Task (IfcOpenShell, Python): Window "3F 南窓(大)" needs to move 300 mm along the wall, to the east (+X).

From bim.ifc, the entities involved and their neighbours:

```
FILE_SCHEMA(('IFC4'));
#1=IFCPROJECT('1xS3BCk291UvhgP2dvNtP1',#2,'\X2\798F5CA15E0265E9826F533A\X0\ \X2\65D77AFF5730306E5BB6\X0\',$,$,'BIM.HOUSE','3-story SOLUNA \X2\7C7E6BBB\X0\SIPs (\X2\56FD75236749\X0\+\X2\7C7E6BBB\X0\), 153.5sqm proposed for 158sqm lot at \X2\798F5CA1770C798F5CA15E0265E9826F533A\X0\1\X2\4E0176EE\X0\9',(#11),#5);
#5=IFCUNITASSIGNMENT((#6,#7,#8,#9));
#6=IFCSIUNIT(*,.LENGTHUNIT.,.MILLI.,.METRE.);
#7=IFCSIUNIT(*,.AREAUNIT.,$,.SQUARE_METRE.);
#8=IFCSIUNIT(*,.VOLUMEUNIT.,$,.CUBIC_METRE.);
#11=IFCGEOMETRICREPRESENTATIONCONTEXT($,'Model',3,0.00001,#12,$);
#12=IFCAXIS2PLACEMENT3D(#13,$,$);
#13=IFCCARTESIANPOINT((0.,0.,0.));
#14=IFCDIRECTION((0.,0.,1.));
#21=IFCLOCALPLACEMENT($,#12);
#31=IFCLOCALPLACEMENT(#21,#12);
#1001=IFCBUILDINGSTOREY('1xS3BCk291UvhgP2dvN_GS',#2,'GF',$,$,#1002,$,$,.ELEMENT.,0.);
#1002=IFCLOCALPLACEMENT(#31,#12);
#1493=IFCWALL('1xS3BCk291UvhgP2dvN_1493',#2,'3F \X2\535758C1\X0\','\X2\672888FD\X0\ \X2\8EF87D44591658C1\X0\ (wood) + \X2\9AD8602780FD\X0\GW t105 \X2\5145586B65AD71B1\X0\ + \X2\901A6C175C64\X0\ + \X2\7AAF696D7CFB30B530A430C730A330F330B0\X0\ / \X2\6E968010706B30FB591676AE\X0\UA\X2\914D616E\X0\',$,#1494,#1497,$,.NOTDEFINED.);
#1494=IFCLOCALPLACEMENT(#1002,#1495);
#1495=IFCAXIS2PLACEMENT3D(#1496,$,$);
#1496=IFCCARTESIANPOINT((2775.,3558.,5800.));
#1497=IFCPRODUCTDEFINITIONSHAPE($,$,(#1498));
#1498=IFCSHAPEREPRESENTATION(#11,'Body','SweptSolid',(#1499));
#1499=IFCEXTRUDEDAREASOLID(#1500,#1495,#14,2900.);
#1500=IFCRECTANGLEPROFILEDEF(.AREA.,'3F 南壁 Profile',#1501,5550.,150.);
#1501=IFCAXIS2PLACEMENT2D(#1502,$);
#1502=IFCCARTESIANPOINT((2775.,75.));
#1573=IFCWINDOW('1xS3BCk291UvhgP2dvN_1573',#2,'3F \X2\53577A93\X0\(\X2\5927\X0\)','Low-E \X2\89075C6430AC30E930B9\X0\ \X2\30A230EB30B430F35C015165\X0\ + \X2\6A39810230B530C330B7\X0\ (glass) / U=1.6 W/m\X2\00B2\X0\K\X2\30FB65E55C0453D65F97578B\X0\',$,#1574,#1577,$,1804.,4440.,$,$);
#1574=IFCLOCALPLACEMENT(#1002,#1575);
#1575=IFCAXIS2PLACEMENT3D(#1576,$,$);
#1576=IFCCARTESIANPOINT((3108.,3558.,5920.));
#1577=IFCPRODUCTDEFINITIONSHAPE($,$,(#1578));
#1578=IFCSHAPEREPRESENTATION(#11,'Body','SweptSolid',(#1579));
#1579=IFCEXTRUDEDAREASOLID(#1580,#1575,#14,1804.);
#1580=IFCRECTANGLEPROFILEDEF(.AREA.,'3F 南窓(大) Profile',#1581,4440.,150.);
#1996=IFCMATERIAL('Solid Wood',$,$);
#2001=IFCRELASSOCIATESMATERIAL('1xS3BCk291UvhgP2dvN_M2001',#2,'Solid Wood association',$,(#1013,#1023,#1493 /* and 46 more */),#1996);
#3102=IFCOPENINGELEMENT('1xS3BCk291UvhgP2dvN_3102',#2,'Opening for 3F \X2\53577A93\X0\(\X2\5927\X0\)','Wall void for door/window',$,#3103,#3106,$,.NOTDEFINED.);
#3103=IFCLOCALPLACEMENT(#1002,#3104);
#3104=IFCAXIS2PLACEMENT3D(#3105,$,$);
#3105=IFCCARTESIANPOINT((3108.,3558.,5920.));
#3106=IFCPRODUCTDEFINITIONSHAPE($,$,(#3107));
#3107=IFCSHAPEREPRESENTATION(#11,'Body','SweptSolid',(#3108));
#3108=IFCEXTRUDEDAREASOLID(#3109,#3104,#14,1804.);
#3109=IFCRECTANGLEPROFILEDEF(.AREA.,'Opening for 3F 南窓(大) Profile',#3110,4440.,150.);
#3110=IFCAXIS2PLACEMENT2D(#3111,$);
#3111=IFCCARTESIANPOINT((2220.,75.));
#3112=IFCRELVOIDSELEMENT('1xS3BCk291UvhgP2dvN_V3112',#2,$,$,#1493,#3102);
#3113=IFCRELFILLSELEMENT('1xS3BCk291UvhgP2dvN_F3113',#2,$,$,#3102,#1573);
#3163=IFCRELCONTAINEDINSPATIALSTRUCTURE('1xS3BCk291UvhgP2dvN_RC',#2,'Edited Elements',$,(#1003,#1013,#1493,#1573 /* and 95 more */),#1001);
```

```python
import ifcopenshell
import ifcopenshell.api.geometry
import ifcopenshell.util.placement
import ifcopenshell.util.unit

model = ifcopenshell.open("bim.ifc")
unit_scale = ifcopenshell.util.unit.calculate_unit_scale(model)

window = model.by_guid("1xS3BCk291UvhgP2dvN_1573")
opening = window.FillsVoids[0].RelatingOpeningElement
wall = opening.VoidsElements[0].RelatingBuildingElement

wall_matrix = ifcopenshell.util.placement.get_local_placement(wall.ObjectPlacement)
shift = wall_matrix[:3, 0] * 0.3 / unit_scale
before = ifcopenshell.util.placement.get_local_placement(window.ObjectPlacement)[:3, 3].copy()

# The window is not placed relative to its opening, so move both.
for product in (opening, window):
    matrix = ifcopenshell.util.placement.get_local_placement(product.ObjectPlacement)
    matrix[:3, 3] += shift
    ifcopenshell.api.geometry.edit_object_placement(model, product=product, matrix=matrix, is_si=False)

after = ifcopenshell.util.placement.get_local_placement(window.ObjectPlacement)[:3, 3]
print("window moved by", (after - before).round(3) + 0.0)

model.write("bim-out.ifc")
```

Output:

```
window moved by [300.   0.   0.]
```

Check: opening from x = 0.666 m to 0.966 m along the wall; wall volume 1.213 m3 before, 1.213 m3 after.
